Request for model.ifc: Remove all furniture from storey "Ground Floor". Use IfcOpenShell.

First a look at what the model holds.

```python
import ifcopenshell
import ifcopenshell.util.element

model = ifcopenshell.open("model.ifc")
print(model.schema)
storey = next(s for s in model.by_type("IfcBuildingStorey") if s.Name == "Ground Floor")
furniture = [e for e in ifcopenshell.util.element.get_decomposition(storey) if e.is_a("IfcFurnishingElement")]
seen = {}
for e in furniture:
    element_type = ifcopenshell.util.element.get_type(e)
    name = element_type.Name if element_type not in (None, e) else None
    seen[name] = seen.get(name, 0) + 1
for name, count in sorted(seen.items(), key=str):
    print(count, "x", name)
```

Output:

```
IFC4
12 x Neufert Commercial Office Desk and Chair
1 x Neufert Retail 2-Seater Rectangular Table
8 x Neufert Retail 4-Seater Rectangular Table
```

```python
import ifcopenshell
import ifcopenshell.api.root
import ifcopenshell.util.element

model = ifcopenshell.open("model.ifc")

storey = next(s for s in model.by_type("IfcBuildingStorey") if s.Name == "Ground Floor")
furniture = [e for e in ifcopenshell.util.element.get_decomposition(storey) if e.is_a("IfcFurnishingElement")]

for e in furniture:
    ifcopenshell.api.root.remove_product(model, product=e)
print(len(furniture), "removed")

model.write("model_updated.ifc")
```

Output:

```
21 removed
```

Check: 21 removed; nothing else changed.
